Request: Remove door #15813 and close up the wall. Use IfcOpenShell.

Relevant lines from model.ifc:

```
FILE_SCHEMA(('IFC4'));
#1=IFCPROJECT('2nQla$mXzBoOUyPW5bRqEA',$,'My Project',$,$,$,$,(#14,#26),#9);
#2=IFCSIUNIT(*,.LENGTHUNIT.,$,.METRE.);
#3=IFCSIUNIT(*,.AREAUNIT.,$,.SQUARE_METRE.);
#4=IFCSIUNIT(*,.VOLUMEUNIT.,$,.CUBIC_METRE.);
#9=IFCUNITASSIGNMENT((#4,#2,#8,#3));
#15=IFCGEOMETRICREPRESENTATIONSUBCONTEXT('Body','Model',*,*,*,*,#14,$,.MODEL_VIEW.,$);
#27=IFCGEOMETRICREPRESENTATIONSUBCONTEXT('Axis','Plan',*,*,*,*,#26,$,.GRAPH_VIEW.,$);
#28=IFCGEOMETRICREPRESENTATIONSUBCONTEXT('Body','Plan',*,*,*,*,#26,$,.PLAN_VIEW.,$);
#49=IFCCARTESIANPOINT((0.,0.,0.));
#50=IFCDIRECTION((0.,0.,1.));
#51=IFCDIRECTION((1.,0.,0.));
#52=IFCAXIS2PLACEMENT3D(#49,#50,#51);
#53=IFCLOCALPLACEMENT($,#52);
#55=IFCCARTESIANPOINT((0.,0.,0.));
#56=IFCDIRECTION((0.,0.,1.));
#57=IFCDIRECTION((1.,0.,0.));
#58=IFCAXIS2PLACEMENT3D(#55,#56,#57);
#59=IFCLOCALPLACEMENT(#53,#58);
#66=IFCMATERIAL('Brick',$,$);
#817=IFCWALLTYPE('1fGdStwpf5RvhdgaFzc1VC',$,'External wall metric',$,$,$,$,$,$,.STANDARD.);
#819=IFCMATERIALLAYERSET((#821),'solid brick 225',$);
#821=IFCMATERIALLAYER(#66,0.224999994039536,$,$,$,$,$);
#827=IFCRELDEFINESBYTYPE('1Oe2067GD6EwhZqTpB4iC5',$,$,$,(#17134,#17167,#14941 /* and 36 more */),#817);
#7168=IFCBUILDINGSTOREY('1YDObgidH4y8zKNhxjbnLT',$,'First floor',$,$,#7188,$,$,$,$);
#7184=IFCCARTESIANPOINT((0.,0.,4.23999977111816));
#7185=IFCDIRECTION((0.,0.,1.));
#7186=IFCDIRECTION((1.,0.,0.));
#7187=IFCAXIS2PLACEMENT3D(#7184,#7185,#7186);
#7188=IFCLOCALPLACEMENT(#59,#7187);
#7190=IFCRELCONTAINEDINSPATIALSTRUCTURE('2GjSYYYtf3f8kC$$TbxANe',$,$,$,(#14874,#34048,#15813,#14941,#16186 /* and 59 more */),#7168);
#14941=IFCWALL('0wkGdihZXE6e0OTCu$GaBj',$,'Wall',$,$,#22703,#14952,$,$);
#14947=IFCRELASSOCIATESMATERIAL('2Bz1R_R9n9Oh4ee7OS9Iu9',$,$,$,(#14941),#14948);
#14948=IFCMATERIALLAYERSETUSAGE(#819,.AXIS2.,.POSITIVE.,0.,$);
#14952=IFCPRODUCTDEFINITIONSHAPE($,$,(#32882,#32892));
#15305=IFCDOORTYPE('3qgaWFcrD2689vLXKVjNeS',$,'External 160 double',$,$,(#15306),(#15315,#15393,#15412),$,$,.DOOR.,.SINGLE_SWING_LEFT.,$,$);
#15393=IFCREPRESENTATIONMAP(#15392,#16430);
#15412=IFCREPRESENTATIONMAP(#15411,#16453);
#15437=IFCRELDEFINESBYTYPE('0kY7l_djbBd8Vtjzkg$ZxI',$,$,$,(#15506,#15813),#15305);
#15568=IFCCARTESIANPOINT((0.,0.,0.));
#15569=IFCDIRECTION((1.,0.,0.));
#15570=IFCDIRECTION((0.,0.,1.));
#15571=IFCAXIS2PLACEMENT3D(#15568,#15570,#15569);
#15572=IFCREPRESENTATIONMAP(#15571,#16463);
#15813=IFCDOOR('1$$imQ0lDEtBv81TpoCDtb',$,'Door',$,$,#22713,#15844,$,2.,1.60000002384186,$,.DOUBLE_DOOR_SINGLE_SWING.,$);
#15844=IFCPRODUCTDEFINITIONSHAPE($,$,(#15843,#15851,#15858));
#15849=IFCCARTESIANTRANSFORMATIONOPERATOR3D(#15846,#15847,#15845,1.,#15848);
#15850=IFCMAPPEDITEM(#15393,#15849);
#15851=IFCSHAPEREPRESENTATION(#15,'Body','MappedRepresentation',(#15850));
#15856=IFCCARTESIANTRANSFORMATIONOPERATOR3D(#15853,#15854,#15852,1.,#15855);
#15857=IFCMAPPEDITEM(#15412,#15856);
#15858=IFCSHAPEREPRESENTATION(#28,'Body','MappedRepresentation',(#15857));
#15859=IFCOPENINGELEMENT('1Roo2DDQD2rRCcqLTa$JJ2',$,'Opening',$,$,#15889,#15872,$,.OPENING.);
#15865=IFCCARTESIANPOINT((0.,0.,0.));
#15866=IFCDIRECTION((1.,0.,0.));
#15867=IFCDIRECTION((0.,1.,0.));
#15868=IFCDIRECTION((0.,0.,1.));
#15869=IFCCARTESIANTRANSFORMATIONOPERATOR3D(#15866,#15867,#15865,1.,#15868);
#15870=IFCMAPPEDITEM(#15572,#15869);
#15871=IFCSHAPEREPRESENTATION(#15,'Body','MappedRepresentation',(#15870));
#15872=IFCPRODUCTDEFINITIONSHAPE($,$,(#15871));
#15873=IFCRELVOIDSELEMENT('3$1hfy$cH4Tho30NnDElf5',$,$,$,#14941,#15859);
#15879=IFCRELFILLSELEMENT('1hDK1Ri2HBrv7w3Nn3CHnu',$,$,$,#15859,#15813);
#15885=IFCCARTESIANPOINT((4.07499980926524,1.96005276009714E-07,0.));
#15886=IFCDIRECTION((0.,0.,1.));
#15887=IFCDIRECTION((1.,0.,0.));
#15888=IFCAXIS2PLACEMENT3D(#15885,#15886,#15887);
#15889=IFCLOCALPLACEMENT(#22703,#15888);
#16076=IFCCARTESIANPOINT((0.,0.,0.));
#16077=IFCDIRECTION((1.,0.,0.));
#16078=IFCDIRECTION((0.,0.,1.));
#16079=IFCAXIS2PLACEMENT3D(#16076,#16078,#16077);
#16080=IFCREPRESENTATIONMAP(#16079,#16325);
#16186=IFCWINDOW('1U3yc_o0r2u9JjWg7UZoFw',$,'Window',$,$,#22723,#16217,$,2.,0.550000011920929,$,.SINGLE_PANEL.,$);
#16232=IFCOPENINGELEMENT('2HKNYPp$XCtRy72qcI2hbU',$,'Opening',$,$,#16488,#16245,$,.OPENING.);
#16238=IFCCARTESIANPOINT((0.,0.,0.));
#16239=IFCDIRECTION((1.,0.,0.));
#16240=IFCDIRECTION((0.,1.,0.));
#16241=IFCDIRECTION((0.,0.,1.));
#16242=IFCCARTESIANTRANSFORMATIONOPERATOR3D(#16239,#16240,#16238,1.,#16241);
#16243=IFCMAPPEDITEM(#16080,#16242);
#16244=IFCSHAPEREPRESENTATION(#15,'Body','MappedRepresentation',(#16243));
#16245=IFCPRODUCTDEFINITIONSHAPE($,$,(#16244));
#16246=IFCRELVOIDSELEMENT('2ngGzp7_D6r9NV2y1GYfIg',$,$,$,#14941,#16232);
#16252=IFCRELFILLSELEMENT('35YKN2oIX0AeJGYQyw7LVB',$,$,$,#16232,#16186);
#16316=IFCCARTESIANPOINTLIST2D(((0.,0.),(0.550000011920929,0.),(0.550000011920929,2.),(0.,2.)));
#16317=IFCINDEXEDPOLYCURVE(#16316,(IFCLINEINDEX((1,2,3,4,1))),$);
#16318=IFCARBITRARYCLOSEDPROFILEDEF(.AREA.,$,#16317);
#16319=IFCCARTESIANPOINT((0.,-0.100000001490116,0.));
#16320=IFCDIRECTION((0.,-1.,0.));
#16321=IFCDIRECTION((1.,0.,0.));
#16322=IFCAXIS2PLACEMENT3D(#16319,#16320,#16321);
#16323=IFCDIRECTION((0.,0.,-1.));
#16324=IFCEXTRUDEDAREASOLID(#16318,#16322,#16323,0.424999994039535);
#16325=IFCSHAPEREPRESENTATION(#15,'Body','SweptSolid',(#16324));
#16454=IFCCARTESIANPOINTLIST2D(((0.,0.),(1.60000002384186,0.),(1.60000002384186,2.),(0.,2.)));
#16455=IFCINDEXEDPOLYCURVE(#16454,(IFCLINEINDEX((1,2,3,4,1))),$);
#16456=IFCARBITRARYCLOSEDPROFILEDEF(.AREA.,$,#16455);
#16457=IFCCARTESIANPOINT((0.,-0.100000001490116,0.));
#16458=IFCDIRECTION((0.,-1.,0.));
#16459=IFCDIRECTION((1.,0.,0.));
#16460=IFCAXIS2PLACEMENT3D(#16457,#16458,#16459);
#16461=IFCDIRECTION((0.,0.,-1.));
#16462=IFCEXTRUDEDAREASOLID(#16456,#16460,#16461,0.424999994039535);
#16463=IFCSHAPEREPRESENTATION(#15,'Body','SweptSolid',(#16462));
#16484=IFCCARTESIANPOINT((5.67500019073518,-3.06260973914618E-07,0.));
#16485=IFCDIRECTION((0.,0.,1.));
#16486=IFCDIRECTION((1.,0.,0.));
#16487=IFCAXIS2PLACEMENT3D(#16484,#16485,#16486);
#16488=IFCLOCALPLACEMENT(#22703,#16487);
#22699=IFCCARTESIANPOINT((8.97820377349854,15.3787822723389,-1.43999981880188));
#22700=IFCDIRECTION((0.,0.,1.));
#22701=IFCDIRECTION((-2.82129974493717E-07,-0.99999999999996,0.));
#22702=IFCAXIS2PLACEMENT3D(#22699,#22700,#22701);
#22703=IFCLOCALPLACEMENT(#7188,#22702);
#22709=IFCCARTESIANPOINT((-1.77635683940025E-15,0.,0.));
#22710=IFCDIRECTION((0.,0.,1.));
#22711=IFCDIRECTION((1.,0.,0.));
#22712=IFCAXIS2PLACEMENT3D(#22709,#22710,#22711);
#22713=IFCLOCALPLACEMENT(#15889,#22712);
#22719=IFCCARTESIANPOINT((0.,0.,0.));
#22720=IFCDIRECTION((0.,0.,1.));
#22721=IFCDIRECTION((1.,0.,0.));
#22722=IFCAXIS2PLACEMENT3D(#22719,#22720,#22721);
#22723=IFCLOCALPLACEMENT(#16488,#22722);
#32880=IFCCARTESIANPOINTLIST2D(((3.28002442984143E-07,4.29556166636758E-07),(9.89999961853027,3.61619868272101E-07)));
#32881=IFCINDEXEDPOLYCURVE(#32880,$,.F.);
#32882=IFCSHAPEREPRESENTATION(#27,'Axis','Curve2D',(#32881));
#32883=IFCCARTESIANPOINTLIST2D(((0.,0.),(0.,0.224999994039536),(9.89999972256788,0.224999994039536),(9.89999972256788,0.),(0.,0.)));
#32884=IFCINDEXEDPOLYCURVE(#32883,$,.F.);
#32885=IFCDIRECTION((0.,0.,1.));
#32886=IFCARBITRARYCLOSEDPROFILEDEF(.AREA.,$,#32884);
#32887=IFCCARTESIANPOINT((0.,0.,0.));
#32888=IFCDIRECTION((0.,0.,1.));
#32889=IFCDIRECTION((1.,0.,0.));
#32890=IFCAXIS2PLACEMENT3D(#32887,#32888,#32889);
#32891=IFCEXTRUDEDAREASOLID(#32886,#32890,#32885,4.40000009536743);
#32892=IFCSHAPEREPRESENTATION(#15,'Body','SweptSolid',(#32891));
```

```python
import ifcopenshell
import ifcopenshell.api.feature
import ifcopenshell.api.root
import ifcopenshell.geom
import ifcopenshell.util.shape

model = ifcopenshell.open("model.ifc")
settings = ifcopenshell.geom.settings()


def volume(element):
    """Net volume in cubic metres, openings subtracted."""
    shape = ifcopenshell.geom.create_shape(settings, element)
    return ifcopenshell.util.shape.get_volume(shape.geometry)


door = model.by_guid("1$$imQ0lDEtBv81TpoCDtb")
opening = door.FillsVoids[0].RelatingOpeningElement
wall = opening.VoidsElements[0].RelatingBuildingElement
before = volume(wall)

ifcopenshell.api.root.remove_product(model, product=door)
ifcopenshell.api.feature.remove_feature(model, feature=opening)

after = volume(wall)

print(f"wall volume {before:.3f} -> {after:.3f} m3")

model.write("model_rev.ifc")
```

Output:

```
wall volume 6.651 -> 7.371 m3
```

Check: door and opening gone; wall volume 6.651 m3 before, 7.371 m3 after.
